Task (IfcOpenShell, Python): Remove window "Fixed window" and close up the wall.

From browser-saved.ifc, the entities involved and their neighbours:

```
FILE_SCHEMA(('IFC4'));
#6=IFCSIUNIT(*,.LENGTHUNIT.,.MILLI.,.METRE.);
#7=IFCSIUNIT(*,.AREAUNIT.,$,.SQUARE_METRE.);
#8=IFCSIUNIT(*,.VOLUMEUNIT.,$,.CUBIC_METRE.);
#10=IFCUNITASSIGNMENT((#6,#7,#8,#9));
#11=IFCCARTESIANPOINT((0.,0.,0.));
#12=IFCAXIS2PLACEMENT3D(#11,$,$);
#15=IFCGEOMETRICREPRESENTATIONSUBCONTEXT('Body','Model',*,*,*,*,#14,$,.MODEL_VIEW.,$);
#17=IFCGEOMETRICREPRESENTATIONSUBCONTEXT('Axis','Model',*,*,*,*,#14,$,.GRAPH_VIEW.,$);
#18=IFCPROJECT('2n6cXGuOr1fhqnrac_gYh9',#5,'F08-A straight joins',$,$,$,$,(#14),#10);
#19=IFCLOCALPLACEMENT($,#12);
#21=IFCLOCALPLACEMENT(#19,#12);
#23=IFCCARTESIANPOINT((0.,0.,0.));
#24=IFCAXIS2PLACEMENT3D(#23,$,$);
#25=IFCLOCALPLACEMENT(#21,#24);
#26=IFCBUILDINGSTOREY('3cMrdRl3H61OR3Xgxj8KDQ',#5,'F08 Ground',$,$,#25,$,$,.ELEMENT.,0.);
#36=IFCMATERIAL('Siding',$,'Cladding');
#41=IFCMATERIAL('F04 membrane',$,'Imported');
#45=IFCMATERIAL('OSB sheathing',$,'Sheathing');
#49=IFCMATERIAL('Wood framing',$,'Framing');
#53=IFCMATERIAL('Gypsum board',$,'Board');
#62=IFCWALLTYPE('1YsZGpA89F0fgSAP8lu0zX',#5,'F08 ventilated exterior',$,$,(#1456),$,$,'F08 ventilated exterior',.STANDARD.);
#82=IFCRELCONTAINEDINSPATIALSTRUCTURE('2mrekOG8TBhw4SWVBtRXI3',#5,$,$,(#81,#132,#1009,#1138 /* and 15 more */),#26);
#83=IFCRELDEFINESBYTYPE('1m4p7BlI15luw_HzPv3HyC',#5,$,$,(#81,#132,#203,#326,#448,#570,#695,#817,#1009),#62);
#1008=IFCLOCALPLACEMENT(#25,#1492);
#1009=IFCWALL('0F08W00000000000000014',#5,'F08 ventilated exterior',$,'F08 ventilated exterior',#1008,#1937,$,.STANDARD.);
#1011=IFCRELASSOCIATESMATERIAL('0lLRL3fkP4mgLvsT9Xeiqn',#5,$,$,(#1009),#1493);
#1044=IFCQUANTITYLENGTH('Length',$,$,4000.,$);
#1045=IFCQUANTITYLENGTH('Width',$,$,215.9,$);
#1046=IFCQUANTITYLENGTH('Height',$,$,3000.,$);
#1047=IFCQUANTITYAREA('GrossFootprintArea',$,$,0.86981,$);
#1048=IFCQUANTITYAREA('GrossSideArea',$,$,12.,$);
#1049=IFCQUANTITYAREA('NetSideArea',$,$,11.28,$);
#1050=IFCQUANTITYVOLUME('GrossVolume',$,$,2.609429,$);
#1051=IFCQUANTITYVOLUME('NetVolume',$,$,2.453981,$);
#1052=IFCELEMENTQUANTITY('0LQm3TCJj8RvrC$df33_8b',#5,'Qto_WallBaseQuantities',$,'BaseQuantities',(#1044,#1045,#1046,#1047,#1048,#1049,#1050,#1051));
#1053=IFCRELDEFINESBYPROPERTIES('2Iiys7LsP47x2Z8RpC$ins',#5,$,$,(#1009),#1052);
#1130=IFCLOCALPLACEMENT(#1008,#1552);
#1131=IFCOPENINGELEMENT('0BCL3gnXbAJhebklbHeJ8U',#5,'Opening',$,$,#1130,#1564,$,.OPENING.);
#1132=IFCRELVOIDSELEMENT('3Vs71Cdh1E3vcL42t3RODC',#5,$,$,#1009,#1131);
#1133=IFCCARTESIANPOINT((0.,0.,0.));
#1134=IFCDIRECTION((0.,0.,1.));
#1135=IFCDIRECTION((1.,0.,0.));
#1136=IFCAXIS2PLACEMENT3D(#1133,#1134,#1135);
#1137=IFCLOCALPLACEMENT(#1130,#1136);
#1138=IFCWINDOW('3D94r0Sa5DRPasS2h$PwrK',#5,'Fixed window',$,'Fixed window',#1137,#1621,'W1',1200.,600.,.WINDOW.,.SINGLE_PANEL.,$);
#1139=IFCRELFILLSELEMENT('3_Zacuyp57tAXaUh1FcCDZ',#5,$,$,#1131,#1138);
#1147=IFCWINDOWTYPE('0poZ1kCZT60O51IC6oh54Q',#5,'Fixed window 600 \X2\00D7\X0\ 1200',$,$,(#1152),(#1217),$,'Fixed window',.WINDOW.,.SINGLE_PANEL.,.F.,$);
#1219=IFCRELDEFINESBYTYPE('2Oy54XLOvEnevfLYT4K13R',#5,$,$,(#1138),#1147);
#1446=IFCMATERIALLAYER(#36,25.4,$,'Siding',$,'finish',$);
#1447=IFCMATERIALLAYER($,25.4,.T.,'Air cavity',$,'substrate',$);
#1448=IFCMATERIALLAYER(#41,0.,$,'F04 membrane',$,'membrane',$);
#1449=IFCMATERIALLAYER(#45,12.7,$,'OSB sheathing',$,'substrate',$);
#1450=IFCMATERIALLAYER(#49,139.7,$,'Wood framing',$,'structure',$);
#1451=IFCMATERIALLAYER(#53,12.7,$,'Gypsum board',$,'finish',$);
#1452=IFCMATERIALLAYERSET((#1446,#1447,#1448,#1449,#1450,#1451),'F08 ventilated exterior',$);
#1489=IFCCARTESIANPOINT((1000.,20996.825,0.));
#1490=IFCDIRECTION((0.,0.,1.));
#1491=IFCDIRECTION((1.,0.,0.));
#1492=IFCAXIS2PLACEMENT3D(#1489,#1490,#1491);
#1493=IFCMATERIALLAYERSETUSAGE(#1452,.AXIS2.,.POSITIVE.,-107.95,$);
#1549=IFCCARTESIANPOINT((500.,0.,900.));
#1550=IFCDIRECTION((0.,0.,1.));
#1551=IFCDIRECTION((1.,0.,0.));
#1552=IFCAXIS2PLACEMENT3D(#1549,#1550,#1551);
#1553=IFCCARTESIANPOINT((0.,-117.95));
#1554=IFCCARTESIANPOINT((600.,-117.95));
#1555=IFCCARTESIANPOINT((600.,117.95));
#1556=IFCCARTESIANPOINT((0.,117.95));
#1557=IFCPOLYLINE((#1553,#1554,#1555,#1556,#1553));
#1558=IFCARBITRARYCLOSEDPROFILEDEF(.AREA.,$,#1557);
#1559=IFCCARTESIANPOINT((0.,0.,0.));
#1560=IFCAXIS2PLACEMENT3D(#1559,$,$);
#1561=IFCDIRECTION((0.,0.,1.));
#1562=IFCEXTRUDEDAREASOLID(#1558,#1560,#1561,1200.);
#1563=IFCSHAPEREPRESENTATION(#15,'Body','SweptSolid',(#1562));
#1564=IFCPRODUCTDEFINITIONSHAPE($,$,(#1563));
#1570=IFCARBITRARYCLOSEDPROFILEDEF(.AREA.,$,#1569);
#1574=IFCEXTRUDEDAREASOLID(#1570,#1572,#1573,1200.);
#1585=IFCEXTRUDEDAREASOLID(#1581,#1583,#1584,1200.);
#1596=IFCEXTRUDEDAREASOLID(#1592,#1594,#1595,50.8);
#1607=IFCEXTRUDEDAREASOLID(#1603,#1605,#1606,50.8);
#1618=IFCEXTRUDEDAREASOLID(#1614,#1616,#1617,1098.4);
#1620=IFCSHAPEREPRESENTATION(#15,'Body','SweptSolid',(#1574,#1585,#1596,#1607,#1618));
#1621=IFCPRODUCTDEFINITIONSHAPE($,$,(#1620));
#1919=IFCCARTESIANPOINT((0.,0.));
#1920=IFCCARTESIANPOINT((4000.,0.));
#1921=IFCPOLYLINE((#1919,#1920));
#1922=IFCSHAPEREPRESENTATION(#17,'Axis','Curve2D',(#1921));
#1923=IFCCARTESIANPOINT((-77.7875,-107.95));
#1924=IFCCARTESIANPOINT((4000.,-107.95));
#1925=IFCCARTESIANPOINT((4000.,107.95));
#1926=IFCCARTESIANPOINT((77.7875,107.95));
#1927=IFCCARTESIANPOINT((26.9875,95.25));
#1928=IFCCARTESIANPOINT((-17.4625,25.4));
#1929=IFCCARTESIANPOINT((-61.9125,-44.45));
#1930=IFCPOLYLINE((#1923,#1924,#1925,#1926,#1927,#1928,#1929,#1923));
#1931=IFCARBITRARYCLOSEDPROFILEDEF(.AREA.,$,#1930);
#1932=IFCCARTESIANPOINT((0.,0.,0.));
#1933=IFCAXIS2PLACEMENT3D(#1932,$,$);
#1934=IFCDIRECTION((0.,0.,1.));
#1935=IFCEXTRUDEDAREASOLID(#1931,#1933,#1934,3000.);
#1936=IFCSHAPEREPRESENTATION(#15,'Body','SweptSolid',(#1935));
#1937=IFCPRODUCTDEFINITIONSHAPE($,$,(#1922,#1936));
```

```python
import ifcopenshell
import ifcopenshell.api.feature
import ifcopenshell.api.pset
import ifcopenshell.api.root
import ifcopenshell.geom
import ifcopenshell.util.element
import ifcopenshell.util.shape
import ifcopenshell.util.unit

model = ifcopenshell.open("browser-saved.ifc")
area_scale = ifcopenshell.util.unit.calculate_unit_scale(model, "AREAUNIT")
volume_scale = ifcopenshell.util.unit.calculate_unit_scale(model, "VOLUMEUNIT")
settings = ifcopenshell.geom.settings()


def volume(element):
    """Net volume in cubic metres, openings subtracted."""
    shape = ifcopenshell.geom.create_shape(settings, element)
    return ifcopenshell.util.shape.get_volume(shape.geometry)


window = model.by_guid("3D94r0Sa5DRPasS2h$PwrK")
opening = window.FillsVoids[0].RelatingOpeningElement
wall = opening.VoidsElements[0].RelatingBuildingElement
before = volume(wall)

ifcopenshell.api.root.remove_product(model, product=window)
ifcopenshell.api.feature.remove_feature(model, feature=opening)

after = volume(wall)
thickness = 0.2159  # wall thickness in metres

# Update the wall's stored quantities.
qto = model.by_id(ifcopenshell.util.element.get_pset(wall, "Qto_WallBaseQuantities", should_inherit=False)["id"])
ifcopenshell.api.pset.edit_qto(model, qto=qto, properties={
    "NetSideArea": after / thickness / area_scale,
    "NetVolume": after / volume_scale,
})

print(f"wall volume {before:.3f} -> {after:.3f} m3")

model.write("browser-saved-out.ifc")
```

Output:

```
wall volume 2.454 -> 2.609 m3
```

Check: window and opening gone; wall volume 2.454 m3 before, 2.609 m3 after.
